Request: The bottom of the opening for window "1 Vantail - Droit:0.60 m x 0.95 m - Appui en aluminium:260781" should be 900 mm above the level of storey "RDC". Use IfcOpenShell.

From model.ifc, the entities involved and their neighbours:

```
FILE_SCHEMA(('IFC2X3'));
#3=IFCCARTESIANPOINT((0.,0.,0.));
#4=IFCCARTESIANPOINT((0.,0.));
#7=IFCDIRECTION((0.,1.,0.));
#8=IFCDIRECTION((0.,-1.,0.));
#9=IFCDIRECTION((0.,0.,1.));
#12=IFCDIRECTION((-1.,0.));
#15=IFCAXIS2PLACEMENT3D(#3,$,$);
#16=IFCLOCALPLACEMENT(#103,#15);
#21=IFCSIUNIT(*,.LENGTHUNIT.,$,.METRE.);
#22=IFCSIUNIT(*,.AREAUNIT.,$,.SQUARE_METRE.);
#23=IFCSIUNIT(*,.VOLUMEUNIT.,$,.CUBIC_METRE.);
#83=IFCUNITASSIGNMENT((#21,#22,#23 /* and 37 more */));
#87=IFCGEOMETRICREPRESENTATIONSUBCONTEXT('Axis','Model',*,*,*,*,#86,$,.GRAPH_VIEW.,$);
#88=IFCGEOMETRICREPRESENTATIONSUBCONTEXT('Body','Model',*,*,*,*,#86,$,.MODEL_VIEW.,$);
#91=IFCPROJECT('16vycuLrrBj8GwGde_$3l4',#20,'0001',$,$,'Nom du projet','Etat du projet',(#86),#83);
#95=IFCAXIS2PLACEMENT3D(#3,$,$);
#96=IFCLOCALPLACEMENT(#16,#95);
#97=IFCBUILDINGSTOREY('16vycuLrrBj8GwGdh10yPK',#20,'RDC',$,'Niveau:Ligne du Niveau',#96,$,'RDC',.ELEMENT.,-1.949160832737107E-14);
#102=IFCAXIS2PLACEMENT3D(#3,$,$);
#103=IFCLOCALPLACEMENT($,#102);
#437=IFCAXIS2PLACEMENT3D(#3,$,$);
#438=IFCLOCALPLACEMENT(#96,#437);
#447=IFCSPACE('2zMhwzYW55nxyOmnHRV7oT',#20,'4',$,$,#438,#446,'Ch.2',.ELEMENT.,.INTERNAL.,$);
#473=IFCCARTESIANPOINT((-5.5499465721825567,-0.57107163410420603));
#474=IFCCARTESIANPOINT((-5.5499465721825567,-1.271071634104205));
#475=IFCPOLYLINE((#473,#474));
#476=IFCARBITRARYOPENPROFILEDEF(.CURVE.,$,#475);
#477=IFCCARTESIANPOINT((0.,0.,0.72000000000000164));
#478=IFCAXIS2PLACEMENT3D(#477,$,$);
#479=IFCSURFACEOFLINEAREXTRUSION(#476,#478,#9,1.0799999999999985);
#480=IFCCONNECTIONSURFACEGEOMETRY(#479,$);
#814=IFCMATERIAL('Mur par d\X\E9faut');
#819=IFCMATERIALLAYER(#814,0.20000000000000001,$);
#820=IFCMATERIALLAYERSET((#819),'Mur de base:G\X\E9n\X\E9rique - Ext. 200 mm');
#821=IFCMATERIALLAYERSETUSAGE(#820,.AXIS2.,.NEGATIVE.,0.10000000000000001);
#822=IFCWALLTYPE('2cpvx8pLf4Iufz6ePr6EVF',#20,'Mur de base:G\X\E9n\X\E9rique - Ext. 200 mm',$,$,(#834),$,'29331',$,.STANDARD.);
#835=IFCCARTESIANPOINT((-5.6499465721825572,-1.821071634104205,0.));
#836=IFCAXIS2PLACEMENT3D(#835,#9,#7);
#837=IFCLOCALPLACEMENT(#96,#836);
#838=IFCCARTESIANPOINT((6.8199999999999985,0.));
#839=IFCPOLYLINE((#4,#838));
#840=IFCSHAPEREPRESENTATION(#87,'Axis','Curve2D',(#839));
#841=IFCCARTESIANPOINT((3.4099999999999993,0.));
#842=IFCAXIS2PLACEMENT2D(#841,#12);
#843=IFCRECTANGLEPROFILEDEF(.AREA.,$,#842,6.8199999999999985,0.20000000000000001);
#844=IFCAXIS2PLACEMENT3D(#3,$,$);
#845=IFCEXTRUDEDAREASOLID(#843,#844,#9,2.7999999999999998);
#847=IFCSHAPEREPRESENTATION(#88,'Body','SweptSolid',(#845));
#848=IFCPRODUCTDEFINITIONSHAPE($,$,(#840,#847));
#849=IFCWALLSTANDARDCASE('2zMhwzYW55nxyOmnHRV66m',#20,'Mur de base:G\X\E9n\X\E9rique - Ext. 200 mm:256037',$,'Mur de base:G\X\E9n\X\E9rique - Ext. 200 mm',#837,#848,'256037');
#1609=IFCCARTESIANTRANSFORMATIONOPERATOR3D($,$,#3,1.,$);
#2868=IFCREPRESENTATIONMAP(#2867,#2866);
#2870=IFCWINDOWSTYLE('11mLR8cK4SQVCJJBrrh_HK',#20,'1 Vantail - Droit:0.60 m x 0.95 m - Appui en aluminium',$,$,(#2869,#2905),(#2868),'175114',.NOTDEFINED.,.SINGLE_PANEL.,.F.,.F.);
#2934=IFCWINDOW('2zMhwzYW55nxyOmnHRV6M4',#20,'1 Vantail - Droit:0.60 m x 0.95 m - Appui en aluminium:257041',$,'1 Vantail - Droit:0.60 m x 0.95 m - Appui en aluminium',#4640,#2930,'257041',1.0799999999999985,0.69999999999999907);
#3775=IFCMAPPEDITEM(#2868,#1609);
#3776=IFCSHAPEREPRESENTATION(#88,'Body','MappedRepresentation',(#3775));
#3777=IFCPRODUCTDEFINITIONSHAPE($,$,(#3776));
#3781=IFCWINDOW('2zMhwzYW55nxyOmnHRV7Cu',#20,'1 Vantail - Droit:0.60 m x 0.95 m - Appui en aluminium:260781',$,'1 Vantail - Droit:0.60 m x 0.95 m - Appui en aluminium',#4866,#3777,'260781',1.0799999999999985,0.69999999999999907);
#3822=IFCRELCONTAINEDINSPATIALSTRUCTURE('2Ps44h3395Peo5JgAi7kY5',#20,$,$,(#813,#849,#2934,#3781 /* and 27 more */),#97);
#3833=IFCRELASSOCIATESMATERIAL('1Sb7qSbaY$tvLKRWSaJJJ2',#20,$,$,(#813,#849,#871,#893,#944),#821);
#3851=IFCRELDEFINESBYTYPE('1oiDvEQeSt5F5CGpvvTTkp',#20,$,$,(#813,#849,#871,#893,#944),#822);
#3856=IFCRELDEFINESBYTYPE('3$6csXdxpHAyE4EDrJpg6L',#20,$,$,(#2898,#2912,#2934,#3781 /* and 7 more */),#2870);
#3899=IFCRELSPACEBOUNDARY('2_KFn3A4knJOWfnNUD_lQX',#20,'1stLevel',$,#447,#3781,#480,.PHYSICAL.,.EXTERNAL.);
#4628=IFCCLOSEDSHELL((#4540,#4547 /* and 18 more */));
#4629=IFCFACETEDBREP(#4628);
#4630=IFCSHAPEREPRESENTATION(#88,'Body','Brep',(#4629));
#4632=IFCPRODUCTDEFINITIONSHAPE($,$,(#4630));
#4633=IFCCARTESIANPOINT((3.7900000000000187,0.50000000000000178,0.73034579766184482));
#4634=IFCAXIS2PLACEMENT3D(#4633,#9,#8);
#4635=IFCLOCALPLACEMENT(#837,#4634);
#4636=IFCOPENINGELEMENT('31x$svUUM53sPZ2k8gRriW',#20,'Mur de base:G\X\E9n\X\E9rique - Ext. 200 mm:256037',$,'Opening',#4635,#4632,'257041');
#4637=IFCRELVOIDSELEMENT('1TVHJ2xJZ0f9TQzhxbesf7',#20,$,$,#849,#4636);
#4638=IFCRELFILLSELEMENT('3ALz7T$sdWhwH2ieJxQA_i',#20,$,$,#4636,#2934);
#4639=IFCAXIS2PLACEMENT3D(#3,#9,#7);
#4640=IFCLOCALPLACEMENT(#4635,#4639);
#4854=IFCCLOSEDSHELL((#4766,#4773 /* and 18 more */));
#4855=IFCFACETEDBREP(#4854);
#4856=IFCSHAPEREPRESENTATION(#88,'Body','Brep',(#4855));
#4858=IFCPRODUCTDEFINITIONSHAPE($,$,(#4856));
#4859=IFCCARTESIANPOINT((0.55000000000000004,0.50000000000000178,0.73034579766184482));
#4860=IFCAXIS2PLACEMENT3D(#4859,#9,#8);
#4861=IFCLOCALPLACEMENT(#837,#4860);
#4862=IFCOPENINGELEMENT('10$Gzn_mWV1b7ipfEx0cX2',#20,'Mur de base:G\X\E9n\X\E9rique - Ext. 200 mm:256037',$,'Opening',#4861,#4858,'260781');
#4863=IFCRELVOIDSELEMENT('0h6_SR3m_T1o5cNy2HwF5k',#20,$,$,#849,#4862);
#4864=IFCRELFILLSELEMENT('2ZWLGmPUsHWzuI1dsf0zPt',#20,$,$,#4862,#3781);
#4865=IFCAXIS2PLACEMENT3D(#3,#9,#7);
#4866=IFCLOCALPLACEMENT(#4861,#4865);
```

```python
import numpy as np
import ifcopenshell
import ifcopenshell.api.geometry
import ifcopenshell.geom
import ifcopenshell.util.element
import ifcopenshell.util.placement
import ifcopenshell.util.shape
import ifcopenshell.util.unit

model = ifcopenshell.open("model.ifc")
unit_scale = ifcopenshell.util.unit.calculate_unit_scale(model)

window = model.by_guid("2zMhwzYW55nxyOmnHRV7Cu")
opening = window.FillsVoids[0].RelatingOpeningElement
storey = ifcopenshell.util.element.get_container(window, ifc_class="IfcBuildingStorey")
level = ifcopenshell.util.placement.get_local_placement(storey.ObjectPlacement)[2, 3]

# The opening's origin need not be at the sill, so measure its lowest point.
shape = ifcopenshell.geom.create_shape(ifcopenshell.geom.settings(), opening)
bottom = ifcopenshell.util.shape.get_shape_bottom_elevation(shape, shape.geometry) / unit_scale
dz = level + 0.9 / unit_scale - bottom

shift = np.array([0.0, 0.0, dz])
# The window is placed relative to its opening, so it follows when the opening moves.
matrix = ifcopenshell.util.placement.get_local_placement(opening.ObjectPlacement)
matrix[:3, 3] += shift
ifcopenshell.api.geometry.edit_object_placement(
    model, product=opening, matrix=matrix, is_si=False, should_transform_children=True
)

# Space boundary surfaces are stored in each space's coordinates; move them too.
for rel in window.ProvidesBoundaries:
    if not rel.ConnectionGeometry:
        continue
    surface = rel.ConnectionGeometry.SurfaceOnRelatingElement
    space_matrix = ifcopenshell.util.placement.get_local_placement(rel.RelatingSpace.ObjectPlacement)
    point = np.array(surface.Position.Location.Coordinates) + space_matrix[:3, :3].T @ shift
    surface.Position = model.createIfcAxis2Placement3D(
        model.createIfcCartesianPoint(point.tolist()), surface.Position.Axis, surface.Position.RefDirection
    )

print(f"moved by {dz * unit_scale:+.3f} m")

model.write("model_rev.ifc")
```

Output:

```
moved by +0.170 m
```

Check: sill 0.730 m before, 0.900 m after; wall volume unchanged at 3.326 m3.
